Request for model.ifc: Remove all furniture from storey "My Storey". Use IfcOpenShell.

First a look at what the model holds.

```python
import ifcopenshell
import ifcopenshell.util.element

model = ifcopenshell.open("model.ifc")
print(model.schema)
storey = next(s for s in model.by_type("IfcBuildingStorey") if s.Name == "My Storey")
furniture = [e for e in ifcopenshell.util.element.get_decomposition(storey) if e.is_a("IfcFurnishingElement")]
seen = {}
for e in furniture:
    element_type = ifcopenshell.util.element.get_type(e)
    name = element_type.Name if element_type not in (None, e) else None
    seen[name] = seen.get(name, 0) + 1
for name, count in sorted(seen.items(), key=str):
    print(count, "x", name)
```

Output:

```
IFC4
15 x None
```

```python
import ifcopenshell
import ifcopenshell.api.root
import ifcopenshell.util.element

model = ifcopenshell.open("model.ifc")

storey = next(s for s in model.by_type("IfcBuildingStorey") if s.Name == "My Storey")
furniture = [e for e in ifcopenshell.util.element.get_decomposition(storey) if e.is_a("IfcFurnishingElement")]

for e in furniture:
    ifcopenshell.api.root.remove_product(model, product=e)
print(len(furniture), "removed")

model.write("model_rev.ifc")
```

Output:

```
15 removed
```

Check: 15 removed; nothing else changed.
